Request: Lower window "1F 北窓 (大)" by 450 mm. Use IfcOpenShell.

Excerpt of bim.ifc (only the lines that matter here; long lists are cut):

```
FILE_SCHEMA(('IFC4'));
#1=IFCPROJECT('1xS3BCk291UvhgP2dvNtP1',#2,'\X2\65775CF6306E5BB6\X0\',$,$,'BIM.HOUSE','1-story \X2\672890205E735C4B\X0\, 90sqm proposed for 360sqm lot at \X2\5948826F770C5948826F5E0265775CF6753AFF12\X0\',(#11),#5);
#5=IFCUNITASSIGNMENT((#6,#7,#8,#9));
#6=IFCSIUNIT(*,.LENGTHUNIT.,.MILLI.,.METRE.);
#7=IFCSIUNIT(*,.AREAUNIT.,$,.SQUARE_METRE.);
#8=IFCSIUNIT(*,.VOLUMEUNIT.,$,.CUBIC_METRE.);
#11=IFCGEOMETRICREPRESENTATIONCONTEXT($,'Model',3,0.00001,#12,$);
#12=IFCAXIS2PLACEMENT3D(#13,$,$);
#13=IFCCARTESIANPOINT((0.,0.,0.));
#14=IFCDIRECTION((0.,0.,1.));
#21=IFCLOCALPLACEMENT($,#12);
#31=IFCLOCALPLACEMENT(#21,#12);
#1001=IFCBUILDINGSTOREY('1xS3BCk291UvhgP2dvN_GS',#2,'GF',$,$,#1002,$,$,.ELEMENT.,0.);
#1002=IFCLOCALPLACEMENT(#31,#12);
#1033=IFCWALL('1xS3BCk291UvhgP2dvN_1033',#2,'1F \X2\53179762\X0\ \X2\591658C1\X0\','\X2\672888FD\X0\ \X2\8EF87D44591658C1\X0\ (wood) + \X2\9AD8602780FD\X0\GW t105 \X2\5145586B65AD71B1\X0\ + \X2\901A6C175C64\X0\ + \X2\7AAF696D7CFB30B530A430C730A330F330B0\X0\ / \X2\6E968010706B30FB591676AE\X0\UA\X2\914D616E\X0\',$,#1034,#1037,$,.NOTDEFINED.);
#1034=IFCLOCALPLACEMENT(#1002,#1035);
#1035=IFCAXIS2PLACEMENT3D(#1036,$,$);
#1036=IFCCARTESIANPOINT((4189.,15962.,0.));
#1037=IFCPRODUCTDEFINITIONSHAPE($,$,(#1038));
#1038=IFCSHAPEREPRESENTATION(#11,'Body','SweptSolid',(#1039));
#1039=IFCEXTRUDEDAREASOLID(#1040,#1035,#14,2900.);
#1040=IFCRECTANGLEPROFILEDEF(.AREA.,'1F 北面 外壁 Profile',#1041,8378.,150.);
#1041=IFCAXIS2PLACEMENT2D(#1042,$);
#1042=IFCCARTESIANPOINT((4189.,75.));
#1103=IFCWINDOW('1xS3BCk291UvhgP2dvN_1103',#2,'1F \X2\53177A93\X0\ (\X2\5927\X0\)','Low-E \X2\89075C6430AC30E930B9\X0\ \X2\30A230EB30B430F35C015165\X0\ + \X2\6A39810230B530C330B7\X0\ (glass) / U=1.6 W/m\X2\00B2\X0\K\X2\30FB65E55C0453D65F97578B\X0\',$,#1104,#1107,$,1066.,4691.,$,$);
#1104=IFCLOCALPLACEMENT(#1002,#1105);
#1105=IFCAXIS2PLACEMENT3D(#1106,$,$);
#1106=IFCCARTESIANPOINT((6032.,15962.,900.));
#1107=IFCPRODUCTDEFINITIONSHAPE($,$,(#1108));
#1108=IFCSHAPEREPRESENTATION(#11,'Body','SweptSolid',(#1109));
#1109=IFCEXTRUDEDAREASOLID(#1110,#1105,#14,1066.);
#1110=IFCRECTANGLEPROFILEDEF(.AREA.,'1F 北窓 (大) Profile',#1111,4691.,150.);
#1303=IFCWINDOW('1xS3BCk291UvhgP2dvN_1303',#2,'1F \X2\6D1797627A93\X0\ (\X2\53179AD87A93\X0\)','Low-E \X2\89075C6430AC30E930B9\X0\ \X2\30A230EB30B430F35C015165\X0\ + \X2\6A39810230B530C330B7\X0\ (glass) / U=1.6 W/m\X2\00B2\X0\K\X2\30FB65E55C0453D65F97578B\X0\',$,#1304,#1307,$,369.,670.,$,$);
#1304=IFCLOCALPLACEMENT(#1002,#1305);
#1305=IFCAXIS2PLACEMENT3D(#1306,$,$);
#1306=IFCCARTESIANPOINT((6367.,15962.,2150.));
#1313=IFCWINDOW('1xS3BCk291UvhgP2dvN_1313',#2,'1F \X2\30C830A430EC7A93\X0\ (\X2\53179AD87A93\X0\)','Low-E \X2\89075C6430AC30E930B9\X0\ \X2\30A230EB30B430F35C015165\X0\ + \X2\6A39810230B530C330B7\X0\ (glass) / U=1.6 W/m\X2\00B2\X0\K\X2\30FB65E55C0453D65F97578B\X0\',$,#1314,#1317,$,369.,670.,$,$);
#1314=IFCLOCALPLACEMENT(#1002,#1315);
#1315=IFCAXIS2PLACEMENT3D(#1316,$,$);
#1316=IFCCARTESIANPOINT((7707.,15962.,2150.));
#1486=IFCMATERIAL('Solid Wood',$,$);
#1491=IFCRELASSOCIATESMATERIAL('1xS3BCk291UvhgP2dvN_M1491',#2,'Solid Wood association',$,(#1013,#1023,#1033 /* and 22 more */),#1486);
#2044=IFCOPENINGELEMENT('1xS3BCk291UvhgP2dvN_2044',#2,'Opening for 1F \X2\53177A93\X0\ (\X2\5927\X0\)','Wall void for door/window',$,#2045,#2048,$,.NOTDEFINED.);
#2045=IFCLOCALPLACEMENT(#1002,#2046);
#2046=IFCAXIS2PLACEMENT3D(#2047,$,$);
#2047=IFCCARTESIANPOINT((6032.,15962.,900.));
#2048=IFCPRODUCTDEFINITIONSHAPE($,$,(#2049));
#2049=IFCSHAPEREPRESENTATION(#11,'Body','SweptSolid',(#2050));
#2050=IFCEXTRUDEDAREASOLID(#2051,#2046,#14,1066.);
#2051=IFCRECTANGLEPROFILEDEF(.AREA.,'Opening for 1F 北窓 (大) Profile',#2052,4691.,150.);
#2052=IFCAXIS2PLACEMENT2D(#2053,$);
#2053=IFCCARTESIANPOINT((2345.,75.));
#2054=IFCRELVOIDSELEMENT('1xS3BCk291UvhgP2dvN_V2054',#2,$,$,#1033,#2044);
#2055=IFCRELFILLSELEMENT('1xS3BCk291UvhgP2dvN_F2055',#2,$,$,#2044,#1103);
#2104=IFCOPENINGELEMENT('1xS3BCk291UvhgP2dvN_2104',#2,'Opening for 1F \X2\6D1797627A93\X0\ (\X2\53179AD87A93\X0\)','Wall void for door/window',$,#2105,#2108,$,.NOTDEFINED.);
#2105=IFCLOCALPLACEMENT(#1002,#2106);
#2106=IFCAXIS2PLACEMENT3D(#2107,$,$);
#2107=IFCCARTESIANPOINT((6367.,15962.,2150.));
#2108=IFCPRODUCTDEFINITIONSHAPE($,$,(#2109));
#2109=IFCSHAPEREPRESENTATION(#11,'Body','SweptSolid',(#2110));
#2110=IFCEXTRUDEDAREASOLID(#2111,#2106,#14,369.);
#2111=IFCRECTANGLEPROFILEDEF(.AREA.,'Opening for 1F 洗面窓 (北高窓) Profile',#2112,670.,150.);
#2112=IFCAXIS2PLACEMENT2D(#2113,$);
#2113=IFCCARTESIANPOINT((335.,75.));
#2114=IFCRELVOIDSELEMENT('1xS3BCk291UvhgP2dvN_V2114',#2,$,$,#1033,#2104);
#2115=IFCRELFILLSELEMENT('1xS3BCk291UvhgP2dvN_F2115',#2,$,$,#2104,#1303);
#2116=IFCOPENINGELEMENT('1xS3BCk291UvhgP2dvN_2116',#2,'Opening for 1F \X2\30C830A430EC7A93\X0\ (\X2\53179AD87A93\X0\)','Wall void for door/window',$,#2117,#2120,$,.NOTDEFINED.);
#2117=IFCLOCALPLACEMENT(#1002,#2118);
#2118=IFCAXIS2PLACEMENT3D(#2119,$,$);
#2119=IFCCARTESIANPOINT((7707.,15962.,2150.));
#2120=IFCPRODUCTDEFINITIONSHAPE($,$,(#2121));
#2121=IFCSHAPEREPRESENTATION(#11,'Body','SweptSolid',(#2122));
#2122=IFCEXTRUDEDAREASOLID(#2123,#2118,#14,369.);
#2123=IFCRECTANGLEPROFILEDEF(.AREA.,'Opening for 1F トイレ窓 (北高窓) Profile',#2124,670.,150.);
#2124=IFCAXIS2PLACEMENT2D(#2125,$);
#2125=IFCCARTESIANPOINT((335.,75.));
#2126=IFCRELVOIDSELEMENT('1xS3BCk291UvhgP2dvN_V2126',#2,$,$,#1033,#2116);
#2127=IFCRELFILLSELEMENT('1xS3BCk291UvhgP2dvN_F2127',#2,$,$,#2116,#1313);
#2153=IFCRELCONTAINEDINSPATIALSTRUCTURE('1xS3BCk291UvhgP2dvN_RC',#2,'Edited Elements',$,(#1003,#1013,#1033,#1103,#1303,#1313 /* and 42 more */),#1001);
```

```python
import numpy as np
import ifcopenshell
import ifcopenshell.api.geometry
import ifcopenshell.util.placement
import ifcopenshell.util.unit

model = ifcopenshell.open("bim.ifc")
unit_scale = ifcopenshell.util.unit.calculate_unit_scale(model)

window = model.by_guid("1xS3BCk291UvhgP2dvN_1103")
opening = window.FillsVoids[0].RelatingOpeningElement
dz = -0.45 / unit_scale

shift = np.array([0.0, 0.0, dz])
# The window is not placed relative to its opening, so move both.
for product in (opening, window):
    matrix = ifcopenshell.util.placement.get_local_placement(product.ObjectPlacement)
    matrix[:3, 3] += shift
    ifcopenshell.api.geometry.edit_object_placement(model, product=product, matrix=matrix, is_si=False)

print(f"moved by {dz * unit_scale:+.3f} m")

model.write("bim-out.ifc")
```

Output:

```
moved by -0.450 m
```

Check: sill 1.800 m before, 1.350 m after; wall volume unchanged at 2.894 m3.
